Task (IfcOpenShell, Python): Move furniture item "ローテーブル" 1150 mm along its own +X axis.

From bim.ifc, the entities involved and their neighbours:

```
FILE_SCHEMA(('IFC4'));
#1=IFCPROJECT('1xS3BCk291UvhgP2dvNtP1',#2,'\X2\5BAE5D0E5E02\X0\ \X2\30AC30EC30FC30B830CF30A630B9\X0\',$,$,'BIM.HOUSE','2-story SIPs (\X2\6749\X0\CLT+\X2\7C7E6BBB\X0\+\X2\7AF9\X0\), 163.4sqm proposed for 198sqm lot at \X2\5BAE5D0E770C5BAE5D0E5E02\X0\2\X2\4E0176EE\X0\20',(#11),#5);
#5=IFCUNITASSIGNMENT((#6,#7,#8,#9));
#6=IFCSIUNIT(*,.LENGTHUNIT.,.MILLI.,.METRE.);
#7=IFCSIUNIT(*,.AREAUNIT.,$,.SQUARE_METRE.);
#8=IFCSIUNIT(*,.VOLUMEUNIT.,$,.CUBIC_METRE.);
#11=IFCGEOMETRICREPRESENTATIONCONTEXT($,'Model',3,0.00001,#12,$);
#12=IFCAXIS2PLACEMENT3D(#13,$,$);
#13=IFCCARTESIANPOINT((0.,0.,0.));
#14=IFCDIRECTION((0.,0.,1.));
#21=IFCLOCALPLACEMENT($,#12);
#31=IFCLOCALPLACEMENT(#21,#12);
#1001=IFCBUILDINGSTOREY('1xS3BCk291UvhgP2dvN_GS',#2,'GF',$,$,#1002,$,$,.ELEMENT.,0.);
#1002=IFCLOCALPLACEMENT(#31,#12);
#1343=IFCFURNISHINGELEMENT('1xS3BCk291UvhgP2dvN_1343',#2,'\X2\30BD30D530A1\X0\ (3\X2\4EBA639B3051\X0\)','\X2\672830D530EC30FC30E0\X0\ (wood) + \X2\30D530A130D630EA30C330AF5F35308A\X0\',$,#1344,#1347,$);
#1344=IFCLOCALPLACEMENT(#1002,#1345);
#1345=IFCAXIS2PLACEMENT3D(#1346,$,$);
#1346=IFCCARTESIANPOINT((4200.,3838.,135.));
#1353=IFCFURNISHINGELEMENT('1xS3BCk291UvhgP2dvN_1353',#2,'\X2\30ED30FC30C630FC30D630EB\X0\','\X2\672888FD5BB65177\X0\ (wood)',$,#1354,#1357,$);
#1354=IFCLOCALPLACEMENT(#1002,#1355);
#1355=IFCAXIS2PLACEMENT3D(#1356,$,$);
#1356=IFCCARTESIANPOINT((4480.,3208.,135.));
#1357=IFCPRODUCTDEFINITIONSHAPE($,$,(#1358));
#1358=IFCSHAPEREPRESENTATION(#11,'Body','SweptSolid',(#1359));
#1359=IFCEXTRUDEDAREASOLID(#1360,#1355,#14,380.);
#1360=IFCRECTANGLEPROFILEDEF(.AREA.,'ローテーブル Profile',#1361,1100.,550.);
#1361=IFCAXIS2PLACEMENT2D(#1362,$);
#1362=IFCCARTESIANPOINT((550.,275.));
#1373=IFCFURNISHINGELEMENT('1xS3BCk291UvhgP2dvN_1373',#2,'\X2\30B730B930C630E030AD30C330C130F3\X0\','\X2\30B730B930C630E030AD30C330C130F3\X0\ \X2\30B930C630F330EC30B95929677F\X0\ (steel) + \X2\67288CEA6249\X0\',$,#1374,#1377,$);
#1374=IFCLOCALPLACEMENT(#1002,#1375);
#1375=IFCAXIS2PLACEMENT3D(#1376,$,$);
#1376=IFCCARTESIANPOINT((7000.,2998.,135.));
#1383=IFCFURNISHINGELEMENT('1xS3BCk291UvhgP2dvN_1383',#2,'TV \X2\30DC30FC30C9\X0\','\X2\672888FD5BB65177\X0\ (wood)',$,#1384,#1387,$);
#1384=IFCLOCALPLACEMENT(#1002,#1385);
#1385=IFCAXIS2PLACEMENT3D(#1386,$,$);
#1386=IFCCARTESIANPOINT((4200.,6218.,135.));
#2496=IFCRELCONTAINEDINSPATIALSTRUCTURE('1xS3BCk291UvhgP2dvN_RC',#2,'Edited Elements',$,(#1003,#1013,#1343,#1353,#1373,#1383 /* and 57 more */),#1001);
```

```python
import ifcopenshell
import ifcopenshell.api.geometry
import ifcopenshell.util.placement
import ifcopenshell.util.unit

model = ifcopenshell.open("bim.ifc")
unit_scale = ifcopenshell.util.unit.calculate_unit_scale(model)

item = model.by_guid("1xS3BCk291UvhgP2dvN_1353")
matrix = ifcopenshell.util.placement.get_local_placement(item.ObjectPlacement)
matrix[:3, 3] += matrix[:3, 0] * 1.15 / unit_scale
ifcopenshell.api.geometry.edit_object_placement(model, product=item, matrix=matrix, is_si=False)

print(ifcopenshell.util.placement.get_local_placement(item.ObjectPlacement).round(3) + 0.0)

model.write("bim_edited.ifc")
```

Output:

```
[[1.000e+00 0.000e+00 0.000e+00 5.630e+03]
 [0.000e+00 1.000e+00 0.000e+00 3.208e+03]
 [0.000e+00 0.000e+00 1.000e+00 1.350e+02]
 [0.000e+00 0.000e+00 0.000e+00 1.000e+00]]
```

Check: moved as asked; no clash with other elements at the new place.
